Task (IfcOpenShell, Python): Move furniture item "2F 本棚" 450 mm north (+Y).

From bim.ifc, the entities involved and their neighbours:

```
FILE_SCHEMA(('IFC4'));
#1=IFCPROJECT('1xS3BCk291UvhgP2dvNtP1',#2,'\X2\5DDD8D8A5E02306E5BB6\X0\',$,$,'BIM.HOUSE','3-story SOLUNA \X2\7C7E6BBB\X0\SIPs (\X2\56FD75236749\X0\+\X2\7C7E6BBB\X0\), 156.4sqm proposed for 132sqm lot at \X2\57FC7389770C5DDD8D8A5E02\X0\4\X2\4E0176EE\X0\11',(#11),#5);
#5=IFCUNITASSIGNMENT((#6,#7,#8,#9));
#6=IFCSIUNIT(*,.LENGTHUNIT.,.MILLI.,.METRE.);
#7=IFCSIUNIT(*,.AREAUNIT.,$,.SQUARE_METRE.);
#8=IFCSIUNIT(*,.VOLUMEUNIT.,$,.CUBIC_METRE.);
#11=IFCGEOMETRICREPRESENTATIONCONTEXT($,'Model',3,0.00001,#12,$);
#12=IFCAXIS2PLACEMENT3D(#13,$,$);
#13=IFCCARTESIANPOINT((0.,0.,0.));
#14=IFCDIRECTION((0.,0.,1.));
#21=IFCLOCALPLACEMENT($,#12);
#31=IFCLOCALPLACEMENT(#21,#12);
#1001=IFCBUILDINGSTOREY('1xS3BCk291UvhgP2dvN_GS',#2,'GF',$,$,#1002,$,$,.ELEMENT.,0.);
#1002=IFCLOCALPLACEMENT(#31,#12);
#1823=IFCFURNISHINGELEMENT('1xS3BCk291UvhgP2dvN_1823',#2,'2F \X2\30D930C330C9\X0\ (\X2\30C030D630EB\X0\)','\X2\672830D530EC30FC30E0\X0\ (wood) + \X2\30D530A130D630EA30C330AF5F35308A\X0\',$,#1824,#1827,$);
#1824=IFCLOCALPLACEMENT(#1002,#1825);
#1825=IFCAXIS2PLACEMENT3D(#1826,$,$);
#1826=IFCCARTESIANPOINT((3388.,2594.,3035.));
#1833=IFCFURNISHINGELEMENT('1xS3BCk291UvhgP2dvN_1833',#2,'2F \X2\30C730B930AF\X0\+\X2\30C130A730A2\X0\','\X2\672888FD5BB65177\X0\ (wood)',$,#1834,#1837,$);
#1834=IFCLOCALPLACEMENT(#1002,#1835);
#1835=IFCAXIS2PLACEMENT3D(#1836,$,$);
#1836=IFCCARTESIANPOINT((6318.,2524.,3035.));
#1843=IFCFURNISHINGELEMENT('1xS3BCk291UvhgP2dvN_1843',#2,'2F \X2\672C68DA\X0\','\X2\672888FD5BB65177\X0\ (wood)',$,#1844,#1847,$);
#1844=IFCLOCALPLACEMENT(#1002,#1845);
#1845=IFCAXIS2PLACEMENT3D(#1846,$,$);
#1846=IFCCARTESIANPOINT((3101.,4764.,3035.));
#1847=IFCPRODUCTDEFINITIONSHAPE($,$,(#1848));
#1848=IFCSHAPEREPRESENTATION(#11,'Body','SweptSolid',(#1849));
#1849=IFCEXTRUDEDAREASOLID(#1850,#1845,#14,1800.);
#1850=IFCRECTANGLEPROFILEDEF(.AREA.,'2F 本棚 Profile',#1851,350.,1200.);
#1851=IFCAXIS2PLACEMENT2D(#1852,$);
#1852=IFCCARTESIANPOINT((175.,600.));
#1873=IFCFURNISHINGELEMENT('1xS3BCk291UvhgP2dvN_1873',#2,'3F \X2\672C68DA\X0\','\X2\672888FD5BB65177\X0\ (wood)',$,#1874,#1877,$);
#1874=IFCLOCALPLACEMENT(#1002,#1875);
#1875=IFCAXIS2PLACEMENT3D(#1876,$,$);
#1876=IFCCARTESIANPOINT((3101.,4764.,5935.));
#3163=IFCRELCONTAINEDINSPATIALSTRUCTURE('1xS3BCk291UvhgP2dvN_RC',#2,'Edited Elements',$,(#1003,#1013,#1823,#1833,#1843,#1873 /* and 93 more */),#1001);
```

```python
import ifcopenshell
import ifcopenshell.api.geometry
import ifcopenshell.util.placement
import ifcopenshell.util.unit

model = ifcopenshell.open("bim.ifc")
unit_scale = ifcopenshell.util.unit.calculate_unit_scale(model)

item = model.by_guid("1xS3BCk291UvhgP2dvN_1843")
matrix = ifcopenshell.util.placement.get_local_placement(item.ObjectPlacement)
matrix[1, 3] += 0.45 / unit_scale
ifcopenshell.api.geometry.edit_object_placement(model, product=item, matrix=matrix, is_si=False)

print(ifcopenshell.util.placement.get_local_placement(item.ObjectPlacement).round(3) + 0.0)

model.write("bim_updated.ifc")
```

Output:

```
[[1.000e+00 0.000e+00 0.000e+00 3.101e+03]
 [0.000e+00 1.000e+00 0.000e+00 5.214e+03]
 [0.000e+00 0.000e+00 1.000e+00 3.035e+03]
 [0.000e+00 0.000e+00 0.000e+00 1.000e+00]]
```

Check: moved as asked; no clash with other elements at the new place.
